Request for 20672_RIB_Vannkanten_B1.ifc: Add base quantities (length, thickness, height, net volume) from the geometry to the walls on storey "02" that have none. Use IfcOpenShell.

First a look at what the model holds.

```python
import ifcopenshell
import ifcopenshell.util.element
import ifcopenshell.util.unit

model = ifcopenshell.open("20672_RIB_Vannkanten_B1.ifc")
print(model.schema)
for unit_type in ("LENGTHUNIT", "AREAUNIT", "VOLUMEUNIT"):
    print(unit_type, ifcopenshell.util.unit.calculate_unit_scale(model, unit_type))
storey = next(s for s in model.by_type("IfcBuildingStorey") if s.Name == "02")
walls = [e for e in ifcopenshell.util.element.get_decomposition(storey) if e.is_a("IfcWall")]
for e in sorted(walls, key=lambda e: e.id()):
    print(e.id(), e.is_a(), e.Name, list(ifcopenshell.util.element.get_psets(e, qtos_only=True)), sep=" | ")
```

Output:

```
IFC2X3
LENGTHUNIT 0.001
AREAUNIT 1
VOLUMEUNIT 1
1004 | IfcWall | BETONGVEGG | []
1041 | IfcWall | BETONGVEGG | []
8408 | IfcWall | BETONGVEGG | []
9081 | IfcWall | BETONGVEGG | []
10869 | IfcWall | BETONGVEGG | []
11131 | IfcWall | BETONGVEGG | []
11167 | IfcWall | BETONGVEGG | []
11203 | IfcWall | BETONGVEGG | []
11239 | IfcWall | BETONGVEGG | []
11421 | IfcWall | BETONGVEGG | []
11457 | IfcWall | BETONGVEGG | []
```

```python
import ifcopenshell
import ifcopenshell.api.pset
import ifcopenshell.geom
import ifcopenshell.util.element
import ifcopenshell.util.shape
import ifcopenshell.util.unit

model = ifcopenshell.open("20672_RIB_Vannkanten_B1.ifc")
unit_scale = ifcopenshell.util.unit.calculate_unit_scale(model)
volume_scale = ifcopenshell.util.unit.calculate_unit_scale(model, "VOLUMEUNIT")
settings = ifcopenshell.geom.settings()

storey = next(s for s in model.by_type("IfcBuildingStorey") if s.Name == "02")
walls = [e for e in ifcopenshell.util.element.get_decomposition(storey) if e.is_a("IfcWall")]

for e in sorted(walls, key=lambda e: e.id()):
    if ifcopenshell.util.element.get_psets(e, qtos_only=True, should_inherit=False):
        continue
    # Geometry comes back in metres, in the element's own axes.
    shape = ifcopenshell.geom.create_shape(settings, e)
    values = {
        "Length": ifcopenshell.util.shape.get_x(shape.geometry) / unit_scale,
        "Width": ifcopenshell.util.shape.get_y(shape.geometry) / unit_scale,
        "Height": ifcopenshell.util.shape.get_z(shape.geometry) / unit_scale,
        "NetVolume": ifcopenshell.util.shape.get_volume(shape.geometry) / volume_scale,
    }
    qto = ifcopenshell.api.pset.add_qto(model, product=e, name="BaseQuantities")
    ifcopenshell.api.pset.edit_qto(model, qto=qto, properties=values)
    print(e.id(), {k: round(v, 3) for k, v in values.items()})

model.write("20672_RIB_Vannkanten_B1_rev.ifc")
```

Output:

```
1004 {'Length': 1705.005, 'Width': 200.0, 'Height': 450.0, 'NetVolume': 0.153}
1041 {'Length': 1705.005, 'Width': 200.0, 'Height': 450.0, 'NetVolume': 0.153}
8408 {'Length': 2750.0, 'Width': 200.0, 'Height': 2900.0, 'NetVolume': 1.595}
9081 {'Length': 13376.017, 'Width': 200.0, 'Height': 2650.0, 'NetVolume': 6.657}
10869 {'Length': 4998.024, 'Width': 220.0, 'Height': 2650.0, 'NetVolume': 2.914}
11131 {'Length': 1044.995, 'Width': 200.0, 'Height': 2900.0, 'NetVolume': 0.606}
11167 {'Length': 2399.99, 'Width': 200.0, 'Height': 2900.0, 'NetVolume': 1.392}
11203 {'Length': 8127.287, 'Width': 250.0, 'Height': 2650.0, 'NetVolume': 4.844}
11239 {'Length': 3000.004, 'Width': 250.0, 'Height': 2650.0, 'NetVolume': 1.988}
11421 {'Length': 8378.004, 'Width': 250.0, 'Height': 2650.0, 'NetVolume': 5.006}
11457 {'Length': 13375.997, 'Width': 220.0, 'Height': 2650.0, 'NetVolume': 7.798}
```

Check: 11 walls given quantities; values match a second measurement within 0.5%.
